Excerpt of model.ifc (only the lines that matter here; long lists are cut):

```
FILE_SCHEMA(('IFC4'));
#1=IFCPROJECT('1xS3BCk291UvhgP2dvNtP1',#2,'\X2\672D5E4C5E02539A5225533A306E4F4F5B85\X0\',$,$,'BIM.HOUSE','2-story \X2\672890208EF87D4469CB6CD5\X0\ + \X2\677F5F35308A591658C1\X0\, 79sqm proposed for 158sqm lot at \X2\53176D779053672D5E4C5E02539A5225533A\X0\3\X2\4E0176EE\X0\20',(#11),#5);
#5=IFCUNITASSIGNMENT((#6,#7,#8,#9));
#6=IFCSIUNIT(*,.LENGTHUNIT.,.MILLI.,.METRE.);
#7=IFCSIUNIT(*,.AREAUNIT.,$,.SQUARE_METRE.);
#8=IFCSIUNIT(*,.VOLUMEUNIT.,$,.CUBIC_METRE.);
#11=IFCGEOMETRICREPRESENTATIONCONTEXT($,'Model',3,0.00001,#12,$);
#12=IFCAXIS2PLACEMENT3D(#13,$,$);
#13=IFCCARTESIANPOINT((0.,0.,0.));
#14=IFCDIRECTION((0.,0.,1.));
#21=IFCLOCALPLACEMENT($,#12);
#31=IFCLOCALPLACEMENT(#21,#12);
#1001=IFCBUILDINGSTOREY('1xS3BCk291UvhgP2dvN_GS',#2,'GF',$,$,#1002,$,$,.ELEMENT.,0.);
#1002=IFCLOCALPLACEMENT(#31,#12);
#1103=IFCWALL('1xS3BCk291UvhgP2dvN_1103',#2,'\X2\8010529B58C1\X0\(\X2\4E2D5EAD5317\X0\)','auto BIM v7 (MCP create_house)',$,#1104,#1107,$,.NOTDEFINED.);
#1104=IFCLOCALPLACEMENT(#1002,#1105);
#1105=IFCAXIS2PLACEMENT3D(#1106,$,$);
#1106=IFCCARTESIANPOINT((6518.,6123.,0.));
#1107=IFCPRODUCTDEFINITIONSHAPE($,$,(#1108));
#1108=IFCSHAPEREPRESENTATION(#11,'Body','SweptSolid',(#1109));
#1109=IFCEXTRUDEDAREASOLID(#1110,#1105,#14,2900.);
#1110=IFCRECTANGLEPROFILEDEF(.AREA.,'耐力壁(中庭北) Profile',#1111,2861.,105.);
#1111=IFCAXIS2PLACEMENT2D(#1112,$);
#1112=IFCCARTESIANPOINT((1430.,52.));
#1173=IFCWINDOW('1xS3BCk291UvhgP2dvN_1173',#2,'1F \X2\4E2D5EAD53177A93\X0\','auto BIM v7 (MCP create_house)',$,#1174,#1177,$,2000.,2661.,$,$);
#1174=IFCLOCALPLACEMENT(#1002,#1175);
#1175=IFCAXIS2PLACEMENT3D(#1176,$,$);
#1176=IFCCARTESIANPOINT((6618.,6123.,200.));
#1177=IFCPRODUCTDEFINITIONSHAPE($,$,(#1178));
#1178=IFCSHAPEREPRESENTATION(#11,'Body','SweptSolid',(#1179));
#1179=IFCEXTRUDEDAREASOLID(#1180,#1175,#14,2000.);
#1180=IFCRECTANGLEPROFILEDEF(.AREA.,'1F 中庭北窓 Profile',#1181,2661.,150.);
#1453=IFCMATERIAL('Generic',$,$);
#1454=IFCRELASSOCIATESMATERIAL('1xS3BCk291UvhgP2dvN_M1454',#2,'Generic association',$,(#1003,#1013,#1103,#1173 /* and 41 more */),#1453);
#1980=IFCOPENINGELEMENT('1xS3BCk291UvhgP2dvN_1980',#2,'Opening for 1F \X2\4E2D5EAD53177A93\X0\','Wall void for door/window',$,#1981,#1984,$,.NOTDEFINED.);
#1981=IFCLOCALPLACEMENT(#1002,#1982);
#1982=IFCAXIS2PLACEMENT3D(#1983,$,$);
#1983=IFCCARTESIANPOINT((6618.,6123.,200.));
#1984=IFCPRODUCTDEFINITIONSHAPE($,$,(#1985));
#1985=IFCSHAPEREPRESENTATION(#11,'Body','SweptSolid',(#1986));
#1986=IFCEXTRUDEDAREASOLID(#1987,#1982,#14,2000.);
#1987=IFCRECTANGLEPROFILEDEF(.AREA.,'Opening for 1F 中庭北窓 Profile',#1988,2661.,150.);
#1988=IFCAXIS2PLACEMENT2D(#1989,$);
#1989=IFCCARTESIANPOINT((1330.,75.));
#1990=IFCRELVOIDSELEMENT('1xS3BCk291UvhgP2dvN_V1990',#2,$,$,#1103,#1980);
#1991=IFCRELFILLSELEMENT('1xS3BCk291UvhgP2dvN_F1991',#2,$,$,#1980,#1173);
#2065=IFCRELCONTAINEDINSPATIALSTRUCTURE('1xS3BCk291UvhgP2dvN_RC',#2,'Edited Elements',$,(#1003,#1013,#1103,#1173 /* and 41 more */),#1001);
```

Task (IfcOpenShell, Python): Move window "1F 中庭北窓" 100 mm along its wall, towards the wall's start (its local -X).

```python
import ifcopenshell
import ifcopenshell.api.geometry
import ifcopenshell.util.placement
import ifcopenshell.util.unit

model = ifcopenshell.open("model.ifc")
unit_scale = ifcopenshell.util.unit.calculate_unit_scale(model)

window = model.by_guid("1xS3BCk291UvhgP2dvN_1173")
opening = window.FillsVoids[0].RelatingOpeningElement
wall = opening.VoidsElements[0].RelatingBuildingElement

wall_matrix = ifcopenshell.util.placement.get_local_placement(wall.ObjectPlacement)
shift = wall_matrix[:3, 0] * -0.1 / unit_scale
before = ifcopenshell.util.placement.get_local_placement(window.ObjectPlacement)[:3, 3].copy()

# The window is not placed relative to its opening, so move both.
for product in (opening, window):
    matrix = ifcopenshell.util.placement.get_local_placement(product.ObjectPlacement)
    matrix[:3, 3] += shift
    ifcopenshell.api.geometry.edit_object_placement(model, product=product, matrix=matrix, is_si=False)

after = ifcopenshell.util.placement.get_local_placement(window.ObjectPlacement)[:3, 3]
print("window moved by", (after - before).round(3) + 0.0)

model.write("model_v2.ifc")
```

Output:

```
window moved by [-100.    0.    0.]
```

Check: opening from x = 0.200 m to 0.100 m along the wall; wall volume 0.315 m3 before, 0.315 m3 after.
